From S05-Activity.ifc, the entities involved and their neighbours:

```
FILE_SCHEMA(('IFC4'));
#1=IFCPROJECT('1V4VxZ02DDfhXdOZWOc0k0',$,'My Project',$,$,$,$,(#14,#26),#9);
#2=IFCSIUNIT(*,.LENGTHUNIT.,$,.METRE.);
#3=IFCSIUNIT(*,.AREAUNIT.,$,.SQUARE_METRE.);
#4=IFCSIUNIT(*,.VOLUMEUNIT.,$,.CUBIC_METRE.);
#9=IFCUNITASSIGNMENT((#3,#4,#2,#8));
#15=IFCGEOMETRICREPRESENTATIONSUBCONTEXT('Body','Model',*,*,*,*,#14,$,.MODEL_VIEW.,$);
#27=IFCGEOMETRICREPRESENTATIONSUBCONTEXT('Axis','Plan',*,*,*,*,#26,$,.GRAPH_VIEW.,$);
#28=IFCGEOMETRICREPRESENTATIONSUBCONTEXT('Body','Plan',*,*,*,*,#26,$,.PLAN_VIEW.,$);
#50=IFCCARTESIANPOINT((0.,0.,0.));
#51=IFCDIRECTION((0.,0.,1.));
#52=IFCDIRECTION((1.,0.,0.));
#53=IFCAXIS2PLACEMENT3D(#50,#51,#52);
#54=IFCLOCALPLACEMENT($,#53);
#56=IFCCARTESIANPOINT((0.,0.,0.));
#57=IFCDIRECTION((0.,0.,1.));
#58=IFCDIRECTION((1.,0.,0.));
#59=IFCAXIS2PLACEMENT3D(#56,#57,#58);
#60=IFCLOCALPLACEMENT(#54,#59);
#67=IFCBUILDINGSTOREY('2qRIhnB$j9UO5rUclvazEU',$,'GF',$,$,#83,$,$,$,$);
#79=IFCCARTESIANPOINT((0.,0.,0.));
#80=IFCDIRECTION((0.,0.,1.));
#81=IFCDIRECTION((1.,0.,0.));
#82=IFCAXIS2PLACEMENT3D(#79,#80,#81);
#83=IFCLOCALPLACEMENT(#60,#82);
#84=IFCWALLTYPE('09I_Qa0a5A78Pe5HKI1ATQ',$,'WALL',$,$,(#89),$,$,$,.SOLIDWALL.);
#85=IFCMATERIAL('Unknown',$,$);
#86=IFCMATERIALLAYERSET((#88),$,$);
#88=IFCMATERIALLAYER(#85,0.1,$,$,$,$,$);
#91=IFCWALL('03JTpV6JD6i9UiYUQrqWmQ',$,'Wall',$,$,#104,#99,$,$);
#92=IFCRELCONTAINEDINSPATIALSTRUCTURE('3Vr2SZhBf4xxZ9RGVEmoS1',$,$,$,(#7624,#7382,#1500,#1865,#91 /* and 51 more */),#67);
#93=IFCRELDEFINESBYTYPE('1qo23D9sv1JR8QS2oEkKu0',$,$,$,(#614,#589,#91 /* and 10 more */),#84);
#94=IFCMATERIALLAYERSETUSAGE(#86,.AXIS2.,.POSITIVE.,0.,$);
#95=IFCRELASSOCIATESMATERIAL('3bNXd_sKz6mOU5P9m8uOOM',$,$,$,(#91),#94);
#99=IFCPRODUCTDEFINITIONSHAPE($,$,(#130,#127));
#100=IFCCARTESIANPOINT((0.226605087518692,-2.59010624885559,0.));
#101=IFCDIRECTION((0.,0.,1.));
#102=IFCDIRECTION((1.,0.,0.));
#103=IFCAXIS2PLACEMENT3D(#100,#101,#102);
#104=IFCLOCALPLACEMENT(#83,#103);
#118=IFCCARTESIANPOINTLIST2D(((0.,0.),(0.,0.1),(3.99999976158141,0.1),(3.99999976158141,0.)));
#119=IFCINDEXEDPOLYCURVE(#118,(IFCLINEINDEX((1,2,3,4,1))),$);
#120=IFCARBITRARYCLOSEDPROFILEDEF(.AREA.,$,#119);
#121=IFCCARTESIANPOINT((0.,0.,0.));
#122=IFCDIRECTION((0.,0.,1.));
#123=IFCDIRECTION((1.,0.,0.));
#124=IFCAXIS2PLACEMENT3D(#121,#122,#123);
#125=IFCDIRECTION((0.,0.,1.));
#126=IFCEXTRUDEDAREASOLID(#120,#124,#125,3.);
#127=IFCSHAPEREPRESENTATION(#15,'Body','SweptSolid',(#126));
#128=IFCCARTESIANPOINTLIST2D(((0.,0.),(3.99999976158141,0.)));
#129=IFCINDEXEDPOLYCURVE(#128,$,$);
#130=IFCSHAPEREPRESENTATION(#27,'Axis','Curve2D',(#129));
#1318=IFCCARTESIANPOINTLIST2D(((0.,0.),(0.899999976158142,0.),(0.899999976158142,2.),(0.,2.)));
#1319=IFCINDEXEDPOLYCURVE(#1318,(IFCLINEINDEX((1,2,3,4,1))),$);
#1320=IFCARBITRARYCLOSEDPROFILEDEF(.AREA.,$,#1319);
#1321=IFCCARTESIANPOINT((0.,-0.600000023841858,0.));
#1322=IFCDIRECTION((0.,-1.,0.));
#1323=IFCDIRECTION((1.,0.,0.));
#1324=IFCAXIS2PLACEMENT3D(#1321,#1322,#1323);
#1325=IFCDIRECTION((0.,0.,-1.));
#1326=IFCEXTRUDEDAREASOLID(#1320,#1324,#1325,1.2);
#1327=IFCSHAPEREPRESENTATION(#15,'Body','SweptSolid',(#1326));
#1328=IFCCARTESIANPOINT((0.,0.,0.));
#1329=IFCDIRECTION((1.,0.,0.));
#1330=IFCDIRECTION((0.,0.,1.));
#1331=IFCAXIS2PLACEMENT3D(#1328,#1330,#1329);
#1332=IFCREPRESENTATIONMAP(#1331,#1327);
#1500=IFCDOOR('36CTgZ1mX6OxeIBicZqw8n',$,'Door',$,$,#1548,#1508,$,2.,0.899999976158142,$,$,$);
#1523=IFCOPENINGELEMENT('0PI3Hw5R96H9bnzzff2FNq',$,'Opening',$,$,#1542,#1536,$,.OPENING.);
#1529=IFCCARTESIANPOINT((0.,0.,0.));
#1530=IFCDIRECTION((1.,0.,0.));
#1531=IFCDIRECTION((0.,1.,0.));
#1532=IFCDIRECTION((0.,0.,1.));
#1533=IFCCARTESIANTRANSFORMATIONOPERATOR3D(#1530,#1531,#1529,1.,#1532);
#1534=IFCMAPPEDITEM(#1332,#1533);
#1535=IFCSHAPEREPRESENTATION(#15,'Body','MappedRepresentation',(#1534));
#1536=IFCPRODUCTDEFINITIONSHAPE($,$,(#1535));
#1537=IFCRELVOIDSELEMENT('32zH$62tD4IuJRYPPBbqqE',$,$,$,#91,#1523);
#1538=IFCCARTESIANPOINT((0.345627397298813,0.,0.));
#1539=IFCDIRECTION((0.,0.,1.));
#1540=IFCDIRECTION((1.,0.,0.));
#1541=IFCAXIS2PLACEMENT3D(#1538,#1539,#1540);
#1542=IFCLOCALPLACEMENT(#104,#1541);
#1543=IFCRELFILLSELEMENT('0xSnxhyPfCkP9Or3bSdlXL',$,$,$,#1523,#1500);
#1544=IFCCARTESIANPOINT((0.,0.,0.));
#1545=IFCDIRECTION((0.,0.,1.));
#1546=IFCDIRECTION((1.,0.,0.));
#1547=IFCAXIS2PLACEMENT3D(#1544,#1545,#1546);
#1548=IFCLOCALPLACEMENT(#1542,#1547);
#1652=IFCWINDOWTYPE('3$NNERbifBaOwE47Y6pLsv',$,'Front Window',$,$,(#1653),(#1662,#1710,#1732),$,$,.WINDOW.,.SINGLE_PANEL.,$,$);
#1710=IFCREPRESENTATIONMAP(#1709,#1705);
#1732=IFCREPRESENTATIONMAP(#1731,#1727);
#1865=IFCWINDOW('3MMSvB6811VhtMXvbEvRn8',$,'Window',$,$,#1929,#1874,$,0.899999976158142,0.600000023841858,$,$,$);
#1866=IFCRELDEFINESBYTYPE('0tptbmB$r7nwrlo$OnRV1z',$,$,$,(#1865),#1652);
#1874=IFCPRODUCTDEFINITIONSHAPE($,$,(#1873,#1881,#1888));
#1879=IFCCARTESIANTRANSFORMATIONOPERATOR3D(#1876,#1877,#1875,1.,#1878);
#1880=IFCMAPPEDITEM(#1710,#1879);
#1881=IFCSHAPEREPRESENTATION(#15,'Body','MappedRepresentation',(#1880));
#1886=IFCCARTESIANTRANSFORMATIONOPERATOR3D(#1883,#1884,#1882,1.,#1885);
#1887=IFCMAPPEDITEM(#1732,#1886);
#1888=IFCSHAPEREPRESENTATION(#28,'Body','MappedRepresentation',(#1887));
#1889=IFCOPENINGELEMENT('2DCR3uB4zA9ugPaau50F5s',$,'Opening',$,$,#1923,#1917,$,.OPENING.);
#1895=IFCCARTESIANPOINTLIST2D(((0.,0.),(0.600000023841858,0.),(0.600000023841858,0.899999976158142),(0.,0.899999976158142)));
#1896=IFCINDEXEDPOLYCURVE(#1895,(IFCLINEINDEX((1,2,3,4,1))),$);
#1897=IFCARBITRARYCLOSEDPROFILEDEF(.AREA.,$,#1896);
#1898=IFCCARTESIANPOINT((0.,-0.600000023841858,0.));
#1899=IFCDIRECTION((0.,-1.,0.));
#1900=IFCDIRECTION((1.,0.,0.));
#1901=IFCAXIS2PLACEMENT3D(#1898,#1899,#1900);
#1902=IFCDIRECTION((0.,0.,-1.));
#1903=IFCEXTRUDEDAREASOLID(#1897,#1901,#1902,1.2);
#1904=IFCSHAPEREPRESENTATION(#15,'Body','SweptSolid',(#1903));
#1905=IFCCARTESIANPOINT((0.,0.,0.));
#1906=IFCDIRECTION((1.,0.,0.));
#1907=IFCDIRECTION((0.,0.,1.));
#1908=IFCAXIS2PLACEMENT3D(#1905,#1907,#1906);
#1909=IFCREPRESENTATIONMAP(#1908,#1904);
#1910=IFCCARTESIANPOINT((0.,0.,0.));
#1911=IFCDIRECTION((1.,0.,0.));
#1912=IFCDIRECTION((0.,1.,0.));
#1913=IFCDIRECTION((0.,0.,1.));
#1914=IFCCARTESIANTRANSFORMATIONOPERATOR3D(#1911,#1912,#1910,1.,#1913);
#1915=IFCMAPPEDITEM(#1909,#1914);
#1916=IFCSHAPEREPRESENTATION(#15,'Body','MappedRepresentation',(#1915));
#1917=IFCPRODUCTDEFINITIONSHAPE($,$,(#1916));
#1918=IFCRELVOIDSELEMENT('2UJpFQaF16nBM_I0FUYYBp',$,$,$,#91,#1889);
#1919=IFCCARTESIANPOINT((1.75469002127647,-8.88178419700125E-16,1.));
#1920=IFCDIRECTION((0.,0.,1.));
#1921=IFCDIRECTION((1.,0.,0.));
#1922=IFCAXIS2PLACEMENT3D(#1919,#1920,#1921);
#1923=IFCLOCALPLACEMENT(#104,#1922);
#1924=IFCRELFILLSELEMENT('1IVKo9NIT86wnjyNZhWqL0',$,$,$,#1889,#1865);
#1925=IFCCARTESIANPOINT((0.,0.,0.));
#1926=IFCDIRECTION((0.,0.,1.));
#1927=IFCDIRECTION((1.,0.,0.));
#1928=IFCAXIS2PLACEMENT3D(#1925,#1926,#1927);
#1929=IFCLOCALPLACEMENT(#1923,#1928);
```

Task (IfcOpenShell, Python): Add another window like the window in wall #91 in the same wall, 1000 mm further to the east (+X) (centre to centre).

```python
import ifcopenshell
import ifcopenshell.api.feature
import ifcopenshell.api.geometry
import ifcopenshell.api.root
import ifcopenshell.geom
import ifcopenshell.util.element
import ifcopenshell.util.placement
import ifcopenshell.util.shape
import ifcopenshell.util.unit

model = ifcopenshell.open("S05-Activity.ifc")
unit_scale = ifcopenshell.util.unit.calculate_unit_scale(model)
settings = ifcopenshell.geom.settings()


def volume(element):
    """Net volume in cubic metres, openings subtracted."""
    shape = ifcopenshell.geom.create_shape(settings, element)
    return ifcopenshell.util.shape.get_volume(shape.geometry)


window = model.by_guid("3MMSvB6811VhtMXvbEvRn8")
opening = window.FillsVoids[0].RelatingOpeningElement
wall = opening.VoidsElements[0].RelatingBuildingElement
before = volume(wall)
shift = ifcopenshell.util.placement.get_local_placement(wall.ObjectPlacement)[:3, 0] * 1 / unit_scale

# copy_class copies the void relationship, type, container and properties, but no geometry.
new_opening = ifcopenshell.api.root.copy_class(model, product=opening)
new_opening.Representation = ifcopenshell.util.element.copy_deep(
    model, opening.Representation, exclude=["IfcGeometricRepresentationContext", "IfcRepresentationMap"]
)
new_window = ifcopenshell.api.root.copy_class(model, product=window)
new_window.Representation = ifcopenshell.util.element.copy_deep(
    model, window.Representation, exclude=["IfcGeometricRepresentationContext", "IfcRepresentationMap"]
)
ifcopenshell.api.feature.add_filling(model, opening=new_opening, element=new_window)

for old, new in ((opening, new_opening), (window, new_window)):
    matrix = ifcopenshell.util.placement.get_local_placement(old.ObjectPlacement)
    matrix[:3, 3] += shift
    ifcopenshell.api.geometry.edit_object_placement(model, product=new, matrix=matrix, is_si=False)

after = volume(wall)

print(f"wall volume {before:.3f} -> {after:.3f} m3")

model.write("S05-Activity_v2.ifc")
```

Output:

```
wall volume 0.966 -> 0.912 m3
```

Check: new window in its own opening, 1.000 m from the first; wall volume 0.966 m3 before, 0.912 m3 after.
